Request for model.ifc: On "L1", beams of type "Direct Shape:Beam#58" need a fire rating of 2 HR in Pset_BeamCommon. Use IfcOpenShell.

First a look at what the model holds.

```python
import ifcopenshell
import ifcopenshell.util.element

model = ifcopenshell.open("model.ifc")
print(model.schema)
storey = next(s for s in model.by_type("IfcBuildingStorey") if s.Name == "L1")
beams = [e for e in ifcopenshell.util.element.get_decomposition(storey) if e.is_a("IfcBeam")]
seen = {}
for e in beams:
    element_type = ifcopenshell.util.element.get_type(e)
    key = (element_type.Name if element_type != e and element_type else None, ifcopenshell.util.element.get_pset(e, "Pset_BeamCommon", "FireRating"))
    seen[key] = seen.get(key, 0) + 1
for (name, value), count in sorted(seen.items(), key=str):
    print(count, "x", name, "|", value)
```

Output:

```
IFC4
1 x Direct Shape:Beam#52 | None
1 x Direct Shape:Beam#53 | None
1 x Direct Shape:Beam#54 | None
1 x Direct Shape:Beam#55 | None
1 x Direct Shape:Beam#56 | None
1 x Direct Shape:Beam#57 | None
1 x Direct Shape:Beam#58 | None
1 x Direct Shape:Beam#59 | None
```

```python
import ifcopenshell
import ifcopenshell.api.pset
import ifcopenshell.util.element

model = ifcopenshell.open("model.ifc")

storey = next(s for s in model.by_type("IfcBuildingStorey") if s.Name == "L1")
beams = [e for e in ifcopenshell.util.element.get_decomposition(storey) if e.is_a("IfcBeam")]

count = 0
for e in beams:
    element_type = ifcopenshell.util.element.get_type(e)
    if element_type in (None, e) or element_type.Name != "Direct Shape:Beam#58":
        continue
    # add_pset returns the element's existing set when there is one.
    pset = ifcopenshell.api.pset.add_pset(model, product=e, name="Pset_BeamCommon")
    ifcopenshell.api.pset.edit_pset(model, pset=pset, properties={"FireRating": "2 HR"})
    count += 1

print(count, "beams updated")

model.write("model_rev.ifc")
```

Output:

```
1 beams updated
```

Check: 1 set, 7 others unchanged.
